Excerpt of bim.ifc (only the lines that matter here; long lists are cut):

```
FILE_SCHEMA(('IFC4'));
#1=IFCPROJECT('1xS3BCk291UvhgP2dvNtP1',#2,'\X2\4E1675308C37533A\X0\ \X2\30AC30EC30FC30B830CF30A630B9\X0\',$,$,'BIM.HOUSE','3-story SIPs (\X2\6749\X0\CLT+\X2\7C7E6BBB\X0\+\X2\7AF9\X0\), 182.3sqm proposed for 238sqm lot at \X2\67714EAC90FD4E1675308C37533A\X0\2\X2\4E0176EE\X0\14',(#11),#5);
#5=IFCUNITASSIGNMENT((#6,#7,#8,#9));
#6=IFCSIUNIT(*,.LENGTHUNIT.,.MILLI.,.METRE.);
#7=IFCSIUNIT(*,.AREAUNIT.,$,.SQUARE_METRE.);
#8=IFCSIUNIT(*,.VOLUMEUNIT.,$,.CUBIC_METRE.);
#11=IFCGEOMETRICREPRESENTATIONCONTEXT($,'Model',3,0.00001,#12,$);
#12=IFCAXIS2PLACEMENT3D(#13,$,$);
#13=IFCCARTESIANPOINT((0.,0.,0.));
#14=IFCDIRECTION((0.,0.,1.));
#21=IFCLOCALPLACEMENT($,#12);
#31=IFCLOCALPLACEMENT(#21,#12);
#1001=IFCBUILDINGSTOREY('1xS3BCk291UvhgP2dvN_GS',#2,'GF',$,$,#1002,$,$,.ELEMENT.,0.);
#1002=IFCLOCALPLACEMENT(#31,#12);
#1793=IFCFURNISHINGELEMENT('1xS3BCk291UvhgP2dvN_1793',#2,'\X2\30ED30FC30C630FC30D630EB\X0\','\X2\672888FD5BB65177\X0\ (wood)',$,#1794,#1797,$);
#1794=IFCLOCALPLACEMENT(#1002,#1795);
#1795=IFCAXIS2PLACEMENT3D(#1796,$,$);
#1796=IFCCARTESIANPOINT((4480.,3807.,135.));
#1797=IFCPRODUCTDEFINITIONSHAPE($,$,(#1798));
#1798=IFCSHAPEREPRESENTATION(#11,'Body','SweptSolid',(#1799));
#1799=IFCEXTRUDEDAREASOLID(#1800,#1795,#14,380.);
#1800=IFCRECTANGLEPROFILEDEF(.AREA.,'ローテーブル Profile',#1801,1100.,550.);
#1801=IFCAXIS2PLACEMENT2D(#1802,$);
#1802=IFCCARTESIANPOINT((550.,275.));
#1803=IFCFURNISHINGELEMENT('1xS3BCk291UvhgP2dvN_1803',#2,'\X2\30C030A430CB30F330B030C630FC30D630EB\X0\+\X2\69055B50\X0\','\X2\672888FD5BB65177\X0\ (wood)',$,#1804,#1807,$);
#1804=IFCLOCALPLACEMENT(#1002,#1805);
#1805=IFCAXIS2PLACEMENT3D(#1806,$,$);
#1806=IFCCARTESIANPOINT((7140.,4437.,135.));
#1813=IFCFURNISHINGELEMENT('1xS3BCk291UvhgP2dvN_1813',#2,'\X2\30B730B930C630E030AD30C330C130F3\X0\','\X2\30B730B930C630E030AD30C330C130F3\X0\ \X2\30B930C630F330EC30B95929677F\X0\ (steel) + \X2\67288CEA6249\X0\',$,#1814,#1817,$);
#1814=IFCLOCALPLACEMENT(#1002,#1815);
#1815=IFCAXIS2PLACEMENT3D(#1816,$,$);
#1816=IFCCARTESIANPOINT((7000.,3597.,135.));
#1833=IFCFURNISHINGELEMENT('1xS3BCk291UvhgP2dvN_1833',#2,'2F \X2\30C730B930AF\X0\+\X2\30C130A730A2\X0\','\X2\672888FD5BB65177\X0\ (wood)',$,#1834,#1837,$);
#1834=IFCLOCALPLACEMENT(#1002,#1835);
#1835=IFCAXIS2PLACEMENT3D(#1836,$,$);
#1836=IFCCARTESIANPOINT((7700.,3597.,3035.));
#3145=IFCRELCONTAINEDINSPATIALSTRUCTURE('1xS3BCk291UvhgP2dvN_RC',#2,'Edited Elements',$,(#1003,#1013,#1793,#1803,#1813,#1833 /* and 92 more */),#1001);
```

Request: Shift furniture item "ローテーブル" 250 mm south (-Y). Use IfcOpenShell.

```python
import ifcopenshell
import ifcopenshell.api.geometry
import ifcopenshell.util.placement
import ifcopenshell.util.unit

model = ifcopenshell.open("bim.ifc")
unit_scale = ifcopenshell.util.unit.calculate_unit_scale(model)

item = model.by_id(1793)
matrix = ifcopenshell.util.placement.get_local_placement(item.ObjectPlacement)
matrix[1, 3] -= 0.25 / unit_scale
ifcopenshell.api.geometry.edit_object_placement(model, product=item, matrix=matrix, is_si=False)

print(ifcopenshell.util.placement.get_local_placement(item.ObjectPlacement).round(3) + 0.0)

model.write("bim_rev.ifc")
```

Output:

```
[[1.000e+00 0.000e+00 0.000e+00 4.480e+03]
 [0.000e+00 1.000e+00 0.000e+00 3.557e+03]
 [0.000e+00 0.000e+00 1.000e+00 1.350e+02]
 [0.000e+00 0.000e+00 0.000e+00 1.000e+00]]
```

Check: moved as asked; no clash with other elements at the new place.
